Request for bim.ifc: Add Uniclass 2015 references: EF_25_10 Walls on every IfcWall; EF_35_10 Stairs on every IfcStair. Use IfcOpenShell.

First a look at what the model holds.

```python
import ifcopenshell

model = ifcopenshell.open("bim.ifc")
print(model.schema)
print("classifications:", [c.Name for c in model.by_type("IfcClassification")])
for ifc_class in ("IfcDoor", "IfcRoof", "IfcStair", "IfcWall", "IfcWindow"):
    print(ifc_class, len(model.by_type(ifc_class)))
```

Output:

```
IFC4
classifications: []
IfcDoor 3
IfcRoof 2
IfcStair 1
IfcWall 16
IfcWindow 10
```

```python
import ifcopenshell
import ifcopenshell.api.classification

model = ifcopenshell.open("bim.ifc")

system = ifcopenshell.api.classification.add_classification(model, classification="Uniclass 2015")

codes = {
    "IfcWall": ("EF_25_10", "Walls"),
    "IfcStair": ("EF_35_10", "Stairs"),
}
for ifc_class, (code, name) in codes.items():
    products = model.by_type(ifc_class)
    ifcopenshell.api.classification.add_reference(
        model, products=products, classification=system, identification=code, name=name
    )
    print(code, len(products))

model.write("bim-out.ifc")
```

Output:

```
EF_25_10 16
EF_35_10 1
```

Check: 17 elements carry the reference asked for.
